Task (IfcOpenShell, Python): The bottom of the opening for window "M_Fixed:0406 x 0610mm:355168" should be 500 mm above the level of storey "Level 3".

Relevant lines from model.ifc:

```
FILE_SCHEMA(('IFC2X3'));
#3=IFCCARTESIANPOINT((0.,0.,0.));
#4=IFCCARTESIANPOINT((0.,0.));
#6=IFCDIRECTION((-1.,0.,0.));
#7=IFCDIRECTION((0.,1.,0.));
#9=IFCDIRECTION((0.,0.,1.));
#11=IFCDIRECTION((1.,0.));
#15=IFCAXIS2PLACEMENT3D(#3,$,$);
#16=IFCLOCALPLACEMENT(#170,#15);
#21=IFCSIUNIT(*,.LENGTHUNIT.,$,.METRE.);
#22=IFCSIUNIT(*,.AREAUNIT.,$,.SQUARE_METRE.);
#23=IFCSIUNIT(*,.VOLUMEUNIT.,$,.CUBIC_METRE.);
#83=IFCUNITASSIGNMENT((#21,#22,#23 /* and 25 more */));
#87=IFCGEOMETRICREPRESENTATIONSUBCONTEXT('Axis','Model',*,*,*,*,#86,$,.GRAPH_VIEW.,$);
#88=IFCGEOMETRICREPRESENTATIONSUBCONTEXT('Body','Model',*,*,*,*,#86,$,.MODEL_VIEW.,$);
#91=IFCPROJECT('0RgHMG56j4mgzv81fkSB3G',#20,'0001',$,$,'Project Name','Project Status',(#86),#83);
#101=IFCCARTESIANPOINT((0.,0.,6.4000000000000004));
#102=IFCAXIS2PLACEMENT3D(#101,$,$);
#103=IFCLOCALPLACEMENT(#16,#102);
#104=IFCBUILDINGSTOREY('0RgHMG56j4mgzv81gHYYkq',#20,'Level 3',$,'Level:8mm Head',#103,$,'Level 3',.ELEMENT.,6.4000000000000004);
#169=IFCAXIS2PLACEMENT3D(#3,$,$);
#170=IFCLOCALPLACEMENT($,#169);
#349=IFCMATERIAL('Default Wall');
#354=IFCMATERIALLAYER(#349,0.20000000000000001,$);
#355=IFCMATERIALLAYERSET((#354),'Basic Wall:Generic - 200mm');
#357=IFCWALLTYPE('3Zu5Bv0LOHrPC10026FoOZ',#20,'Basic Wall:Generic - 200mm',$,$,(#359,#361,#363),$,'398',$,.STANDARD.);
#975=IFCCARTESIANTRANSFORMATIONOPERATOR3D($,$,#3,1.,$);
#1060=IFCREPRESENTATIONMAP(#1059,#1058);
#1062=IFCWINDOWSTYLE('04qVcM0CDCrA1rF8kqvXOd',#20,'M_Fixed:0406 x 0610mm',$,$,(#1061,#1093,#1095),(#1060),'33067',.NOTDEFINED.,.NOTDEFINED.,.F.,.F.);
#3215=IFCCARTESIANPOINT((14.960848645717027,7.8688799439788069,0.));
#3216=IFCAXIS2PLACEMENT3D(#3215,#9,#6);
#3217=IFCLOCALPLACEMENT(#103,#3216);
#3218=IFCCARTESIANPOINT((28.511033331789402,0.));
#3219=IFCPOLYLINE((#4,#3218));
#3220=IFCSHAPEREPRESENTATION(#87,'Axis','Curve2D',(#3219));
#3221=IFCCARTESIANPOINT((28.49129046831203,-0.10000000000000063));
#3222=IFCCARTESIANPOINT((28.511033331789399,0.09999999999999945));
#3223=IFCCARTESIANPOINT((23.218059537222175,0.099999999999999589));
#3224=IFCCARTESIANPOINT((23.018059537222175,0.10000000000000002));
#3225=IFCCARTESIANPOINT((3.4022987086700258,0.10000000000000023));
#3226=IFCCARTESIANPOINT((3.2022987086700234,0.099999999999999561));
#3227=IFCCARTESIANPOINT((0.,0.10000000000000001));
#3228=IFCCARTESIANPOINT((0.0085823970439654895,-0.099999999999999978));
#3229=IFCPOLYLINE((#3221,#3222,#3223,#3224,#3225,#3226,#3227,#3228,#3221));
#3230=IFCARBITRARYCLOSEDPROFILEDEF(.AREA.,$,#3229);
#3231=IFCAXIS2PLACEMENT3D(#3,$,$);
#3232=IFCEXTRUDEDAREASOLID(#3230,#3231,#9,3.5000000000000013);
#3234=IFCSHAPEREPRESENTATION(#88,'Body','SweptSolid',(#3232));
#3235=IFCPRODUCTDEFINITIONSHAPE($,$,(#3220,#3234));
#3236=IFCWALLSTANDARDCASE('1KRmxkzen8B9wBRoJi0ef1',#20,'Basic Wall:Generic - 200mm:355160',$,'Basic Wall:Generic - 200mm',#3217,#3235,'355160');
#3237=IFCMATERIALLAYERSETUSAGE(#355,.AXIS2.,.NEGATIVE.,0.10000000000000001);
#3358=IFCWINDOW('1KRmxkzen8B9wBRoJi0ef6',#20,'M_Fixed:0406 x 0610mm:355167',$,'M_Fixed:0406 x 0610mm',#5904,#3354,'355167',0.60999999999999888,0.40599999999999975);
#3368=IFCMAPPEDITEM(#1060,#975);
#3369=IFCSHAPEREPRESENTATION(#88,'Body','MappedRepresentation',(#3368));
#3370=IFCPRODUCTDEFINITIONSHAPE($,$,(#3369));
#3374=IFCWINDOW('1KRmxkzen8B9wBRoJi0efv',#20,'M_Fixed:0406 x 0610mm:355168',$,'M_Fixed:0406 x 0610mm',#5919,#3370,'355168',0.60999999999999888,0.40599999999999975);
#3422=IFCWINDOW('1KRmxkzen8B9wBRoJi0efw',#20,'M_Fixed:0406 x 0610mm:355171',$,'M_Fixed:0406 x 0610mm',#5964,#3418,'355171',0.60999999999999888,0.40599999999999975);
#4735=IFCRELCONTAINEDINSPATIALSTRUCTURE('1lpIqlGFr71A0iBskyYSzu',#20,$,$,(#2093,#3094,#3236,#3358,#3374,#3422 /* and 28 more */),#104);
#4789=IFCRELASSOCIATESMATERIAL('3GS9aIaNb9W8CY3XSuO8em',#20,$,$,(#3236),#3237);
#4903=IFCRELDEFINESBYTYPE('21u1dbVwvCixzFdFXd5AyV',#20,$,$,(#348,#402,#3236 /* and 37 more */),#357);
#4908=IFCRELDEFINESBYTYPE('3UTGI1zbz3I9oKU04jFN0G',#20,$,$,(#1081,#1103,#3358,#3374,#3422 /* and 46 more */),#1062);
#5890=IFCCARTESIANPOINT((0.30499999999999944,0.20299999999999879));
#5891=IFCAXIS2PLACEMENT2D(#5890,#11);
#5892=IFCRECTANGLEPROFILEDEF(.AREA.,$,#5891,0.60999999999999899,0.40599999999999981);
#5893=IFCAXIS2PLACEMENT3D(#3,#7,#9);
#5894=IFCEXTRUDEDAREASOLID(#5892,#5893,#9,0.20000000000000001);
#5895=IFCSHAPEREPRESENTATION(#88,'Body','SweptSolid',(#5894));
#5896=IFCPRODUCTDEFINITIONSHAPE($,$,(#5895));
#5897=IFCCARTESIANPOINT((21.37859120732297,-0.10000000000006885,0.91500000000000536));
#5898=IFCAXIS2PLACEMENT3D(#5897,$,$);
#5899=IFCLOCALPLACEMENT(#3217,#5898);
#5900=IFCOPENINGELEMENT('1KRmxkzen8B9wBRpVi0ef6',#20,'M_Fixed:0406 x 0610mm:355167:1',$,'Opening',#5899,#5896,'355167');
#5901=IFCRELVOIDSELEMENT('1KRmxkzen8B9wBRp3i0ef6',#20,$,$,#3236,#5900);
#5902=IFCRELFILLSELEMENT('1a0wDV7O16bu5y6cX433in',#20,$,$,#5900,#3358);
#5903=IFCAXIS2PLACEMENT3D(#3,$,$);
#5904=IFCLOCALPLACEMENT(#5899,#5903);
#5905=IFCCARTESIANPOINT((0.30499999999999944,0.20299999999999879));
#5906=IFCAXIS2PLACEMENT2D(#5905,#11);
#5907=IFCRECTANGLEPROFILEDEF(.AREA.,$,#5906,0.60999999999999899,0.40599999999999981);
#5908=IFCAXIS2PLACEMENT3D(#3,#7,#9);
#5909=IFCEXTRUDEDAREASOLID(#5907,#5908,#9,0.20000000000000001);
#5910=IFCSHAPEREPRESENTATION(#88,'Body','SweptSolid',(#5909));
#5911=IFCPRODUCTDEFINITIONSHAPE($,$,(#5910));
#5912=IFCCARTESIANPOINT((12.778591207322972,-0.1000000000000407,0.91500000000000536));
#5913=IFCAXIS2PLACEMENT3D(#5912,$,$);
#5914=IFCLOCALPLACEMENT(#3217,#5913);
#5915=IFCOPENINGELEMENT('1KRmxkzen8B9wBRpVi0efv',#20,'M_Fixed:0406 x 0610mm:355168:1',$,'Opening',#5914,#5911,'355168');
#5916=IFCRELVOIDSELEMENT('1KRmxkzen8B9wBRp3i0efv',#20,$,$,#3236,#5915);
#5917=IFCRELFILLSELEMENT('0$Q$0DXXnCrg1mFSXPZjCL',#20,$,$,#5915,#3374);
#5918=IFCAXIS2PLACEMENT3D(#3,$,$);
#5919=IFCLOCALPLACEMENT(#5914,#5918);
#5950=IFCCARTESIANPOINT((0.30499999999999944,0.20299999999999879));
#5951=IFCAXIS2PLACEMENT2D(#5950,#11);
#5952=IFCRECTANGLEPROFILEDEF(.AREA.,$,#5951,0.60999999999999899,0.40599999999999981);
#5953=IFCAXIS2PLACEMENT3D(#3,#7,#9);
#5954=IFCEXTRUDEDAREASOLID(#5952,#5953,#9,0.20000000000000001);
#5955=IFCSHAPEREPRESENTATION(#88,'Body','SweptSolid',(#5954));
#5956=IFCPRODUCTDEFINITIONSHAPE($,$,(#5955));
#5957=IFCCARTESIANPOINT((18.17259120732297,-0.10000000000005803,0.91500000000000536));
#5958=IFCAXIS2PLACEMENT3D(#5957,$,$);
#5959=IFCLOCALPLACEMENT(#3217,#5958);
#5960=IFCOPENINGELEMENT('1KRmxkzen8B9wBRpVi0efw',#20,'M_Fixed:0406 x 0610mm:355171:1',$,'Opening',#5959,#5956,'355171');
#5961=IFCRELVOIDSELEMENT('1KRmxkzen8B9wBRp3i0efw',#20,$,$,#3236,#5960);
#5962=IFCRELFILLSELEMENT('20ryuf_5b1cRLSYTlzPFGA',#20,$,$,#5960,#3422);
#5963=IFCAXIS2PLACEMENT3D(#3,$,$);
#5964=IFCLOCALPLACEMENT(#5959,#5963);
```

```python
import numpy as np
import ifcopenshell
import ifcopenshell.api.geometry
import ifcopenshell.geom
import ifcopenshell.util.element
import ifcopenshell.util.placement
import ifcopenshell.util.shape
import ifcopenshell.util.unit

model = ifcopenshell.open("model.ifc")
unit_scale = ifcopenshell.util.unit.calculate_unit_scale(model)

window = model.by_id(3374)
opening = window.FillsVoids[0].RelatingOpeningElement
storey = ifcopenshell.util.element.get_container(window, ifc_class="IfcBuildingStorey")
level = ifcopenshell.util.placement.get_local_placement(storey.ObjectPlacement)[2, 3]

# The opening's origin need not be at the sill, so measure its lowest point.
shape = ifcopenshell.geom.create_shape(ifcopenshell.geom.settings(), opening)
bottom = ifcopenshell.util.shape.get_shape_bottom_elevation(shape, shape.geometry) / unit_scale
dz = level + 0.5 / unit_scale - bottom

shift = np.array([0.0, 0.0, dz])
# The window is placed relative to its opening, so it follows when the opening moves.
matrix = ifcopenshell.util.placement.get_local_placement(opening.ObjectPlacement)
matrix[:3, 3] += shift
ifcopenshell.api.geometry.edit_object_placement(
    model, product=opening, matrix=matrix, is_si=False, should_transform_children=True
)

print(f"moved by {dz * unit_scale:+.3f} m")

model.write("model_edited.ifc")
```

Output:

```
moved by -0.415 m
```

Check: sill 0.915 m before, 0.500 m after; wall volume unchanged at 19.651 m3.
